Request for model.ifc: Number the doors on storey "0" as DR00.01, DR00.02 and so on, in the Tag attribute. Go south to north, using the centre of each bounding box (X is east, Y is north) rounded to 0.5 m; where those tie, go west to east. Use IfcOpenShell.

First a look at what the model holds.

```python
import ifcopenshell
import ifcopenshell.util.element
import ifcopenshell.util.placement

model = ifcopenshell.open("model.ifc")
print(model.schema)
storey = next(s for s in model.by_type("IfcBuildingStorey") if s.Name == "0")
doors = [e for e in ifcopenshell.util.element.get_decomposition(storey) if e.is_a("IfcDoor")]
for e in sorted(doors, key=lambda e: e.id()):
    origin = ifcopenshell.util.placement.get_local_placement(e.ObjectPlacement)[:3, 3]
    print(e.id(), e.Tag, e.Name, origin.round(2) + 0.0, sep=" | ")
```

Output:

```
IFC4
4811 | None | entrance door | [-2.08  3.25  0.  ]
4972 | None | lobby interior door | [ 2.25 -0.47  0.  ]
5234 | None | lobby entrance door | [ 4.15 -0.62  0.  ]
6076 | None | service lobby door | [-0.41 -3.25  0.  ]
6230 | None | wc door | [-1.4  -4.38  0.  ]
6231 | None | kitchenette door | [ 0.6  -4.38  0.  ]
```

```python
import ifcopenshell
import ifcopenshell.geom
import ifcopenshell.util.element
import ifcopenshell.util.shape

model = ifcopenshell.open("model.ifc")
settings = ifcopenshell.geom.settings()
settings.set("use-world-coords", True)


def centre(element):
    shape = ifcopenshell.geom.create_shape(settings, element)
    return ifcopenshell.util.shape.get_bbox_centroid(shape.geometry)


storey = next(s for s in model.by_type("IfcBuildingStorey") if s.Name == "0")
doors = [e for e in ifcopenshell.util.element.get_decomposition(storey) if e.is_a("IfcDoor")]

# Insertion points can sit at a corner or the storey origin, so sort by the geometry (in metres).
centres = {e: centre(e) for e in doors}
doors.sort(key=lambda e: (round(centres[e][1] / 0.5), centres[e][0]))

for i, e in enumerate(doors, start=1):
    number = f"DR00.{i:02d}"
    e.Tag = number
    print(e.id(), number)

model.write("model_edited.ifc")
```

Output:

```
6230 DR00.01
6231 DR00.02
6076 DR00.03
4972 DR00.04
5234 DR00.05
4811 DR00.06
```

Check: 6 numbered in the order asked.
